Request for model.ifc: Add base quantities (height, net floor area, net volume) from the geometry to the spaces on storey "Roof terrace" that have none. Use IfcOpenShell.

First a look at what the model holds.

```python
import ifcopenshell
import ifcopenshell.util.element
import ifcopenshell.util.unit

model = ifcopenshell.open("model.ifc")
print(model.schema)
for unit_type in ("LENGTHUNIT", "AREAUNIT", "VOLUMEUNIT"):
    print(unit_type, ifcopenshell.util.unit.calculate_unit_scale(model, unit_type))
storey = next(s for s in model.by_type("IfcBuildingStorey") if s.Name == "Roof terrace")
spaces = [e for e in ifcopenshell.util.element.get_decomposition(storey) if e.is_a("IfcSpace")]
for e in sorted(spaces, key=lambda e: e.id()):
    print(e.id(), e.is_a(), e.Name, list(ifcopenshell.util.element.get_psets(e, qtos_only=True)), sep=" | ")
```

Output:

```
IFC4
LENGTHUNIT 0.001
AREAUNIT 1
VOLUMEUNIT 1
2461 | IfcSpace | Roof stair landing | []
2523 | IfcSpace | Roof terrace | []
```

```python
import ifcopenshell
import ifcopenshell.api.pset
import ifcopenshell.geom
import ifcopenshell.util.element
import ifcopenshell.util.shape
import ifcopenshell.util.unit

model = ifcopenshell.open("model.ifc")
unit_scale = ifcopenshell.util.unit.calculate_unit_scale(model)
area_scale = ifcopenshell.util.unit.calculate_unit_scale(model, "AREAUNIT")
volume_scale = ifcopenshell.util.unit.calculate_unit_scale(model, "VOLUMEUNIT")
settings = ifcopenshell.geom.settings()

storey = next(s for s in model.by_type("IfcBuildingStorey") if s.Name == "Roof terrace")
spaces = [e for e in ifcopenshell.util.element.get_decomposition(storey) if e.is_a("IfcSpace")]

for e in sorted(spaces, key=lambda e: e.id()):
    if ifcopenshell.util.element.get_psets(e, qtos_only=True, should_inherit=False):
        continue
    # Geometry comes back in metres, in the element's own axes.
    shape = ifcopenshell.geom.create_shape(settings, e)
    values = {
        "Height": ifcopenshell.util.shape.get_z(shape.geometry) / unit_scale,
        "NetFloorArea": ifcopenshell.util.shape.get_footprint_area(shape.geometry) / area_scale,
        "NetVolume": ifcopenshell.util.shape.get_volume(shape.geometry) / volume_scale,
    }
    qto = ifcopenshell.api.pset.add_qto(model, product=e, name="Qto_SpaceBaseQuantities")
    ifcopenshell.api.pset.edit_qto(model, qto=qto, properties=values)
    print(e.id(), {k: round(v, 3) for k, v in values.items()})

model.write("model_rev.ifc")
```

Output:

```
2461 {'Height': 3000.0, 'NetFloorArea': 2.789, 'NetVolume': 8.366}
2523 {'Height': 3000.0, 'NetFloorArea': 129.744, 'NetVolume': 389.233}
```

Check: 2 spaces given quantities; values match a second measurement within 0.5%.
